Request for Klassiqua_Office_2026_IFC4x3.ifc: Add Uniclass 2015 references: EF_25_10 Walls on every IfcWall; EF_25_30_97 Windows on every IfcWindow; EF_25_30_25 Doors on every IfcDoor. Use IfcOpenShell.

First a look at what the model holds.

```python
import ifcopenshell

model = ifcopenshell.open("Klassiqua_Office_2026_IFC4x3.ifc")
print(model.schema)
print("classifications:", [c.Name for c in model.by_type("IfcClassification")])
for ifc_class in ("IfcDoor", "IfcRoof", "IfcStair", "IfcWall", "IfcWindow"):
    print(ifc_class, len(model.by_type(ifc_class)))
```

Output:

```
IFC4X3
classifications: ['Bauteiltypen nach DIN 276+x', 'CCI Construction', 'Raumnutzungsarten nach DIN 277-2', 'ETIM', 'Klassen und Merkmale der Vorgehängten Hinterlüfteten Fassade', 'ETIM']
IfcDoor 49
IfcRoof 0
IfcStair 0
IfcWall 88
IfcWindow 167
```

```python
import ifcopenshell
import ifcopenshell.api.classification

model = ifcopenshell.open("Klassiqua_Office_2026_IFC4x3.ifc")

system = ifcopenshell.api.classification.add_classification(model, classification="Uniclass 2015")

codes = {
    "IfcWall": ("EF_25_10", "Walls"),
    "IfcWindow": ("EF_25_30_97", "Windows"),
    "IfcDoor": ("EF_25_30_25", "Doors"),
}
for ifc_class, (code, name) in codes.items():
    products = model.by_type(ifc_class)
    ifcopenshell.api.classification.add_reference(
        model, products=products, classification=system, identification=code, name=name
    )
    print(code, len(products))

model.write("Klassiqua_Office_2026_IFC4x3_v2.ifc")
```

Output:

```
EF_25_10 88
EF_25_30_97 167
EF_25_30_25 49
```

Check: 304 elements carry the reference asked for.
